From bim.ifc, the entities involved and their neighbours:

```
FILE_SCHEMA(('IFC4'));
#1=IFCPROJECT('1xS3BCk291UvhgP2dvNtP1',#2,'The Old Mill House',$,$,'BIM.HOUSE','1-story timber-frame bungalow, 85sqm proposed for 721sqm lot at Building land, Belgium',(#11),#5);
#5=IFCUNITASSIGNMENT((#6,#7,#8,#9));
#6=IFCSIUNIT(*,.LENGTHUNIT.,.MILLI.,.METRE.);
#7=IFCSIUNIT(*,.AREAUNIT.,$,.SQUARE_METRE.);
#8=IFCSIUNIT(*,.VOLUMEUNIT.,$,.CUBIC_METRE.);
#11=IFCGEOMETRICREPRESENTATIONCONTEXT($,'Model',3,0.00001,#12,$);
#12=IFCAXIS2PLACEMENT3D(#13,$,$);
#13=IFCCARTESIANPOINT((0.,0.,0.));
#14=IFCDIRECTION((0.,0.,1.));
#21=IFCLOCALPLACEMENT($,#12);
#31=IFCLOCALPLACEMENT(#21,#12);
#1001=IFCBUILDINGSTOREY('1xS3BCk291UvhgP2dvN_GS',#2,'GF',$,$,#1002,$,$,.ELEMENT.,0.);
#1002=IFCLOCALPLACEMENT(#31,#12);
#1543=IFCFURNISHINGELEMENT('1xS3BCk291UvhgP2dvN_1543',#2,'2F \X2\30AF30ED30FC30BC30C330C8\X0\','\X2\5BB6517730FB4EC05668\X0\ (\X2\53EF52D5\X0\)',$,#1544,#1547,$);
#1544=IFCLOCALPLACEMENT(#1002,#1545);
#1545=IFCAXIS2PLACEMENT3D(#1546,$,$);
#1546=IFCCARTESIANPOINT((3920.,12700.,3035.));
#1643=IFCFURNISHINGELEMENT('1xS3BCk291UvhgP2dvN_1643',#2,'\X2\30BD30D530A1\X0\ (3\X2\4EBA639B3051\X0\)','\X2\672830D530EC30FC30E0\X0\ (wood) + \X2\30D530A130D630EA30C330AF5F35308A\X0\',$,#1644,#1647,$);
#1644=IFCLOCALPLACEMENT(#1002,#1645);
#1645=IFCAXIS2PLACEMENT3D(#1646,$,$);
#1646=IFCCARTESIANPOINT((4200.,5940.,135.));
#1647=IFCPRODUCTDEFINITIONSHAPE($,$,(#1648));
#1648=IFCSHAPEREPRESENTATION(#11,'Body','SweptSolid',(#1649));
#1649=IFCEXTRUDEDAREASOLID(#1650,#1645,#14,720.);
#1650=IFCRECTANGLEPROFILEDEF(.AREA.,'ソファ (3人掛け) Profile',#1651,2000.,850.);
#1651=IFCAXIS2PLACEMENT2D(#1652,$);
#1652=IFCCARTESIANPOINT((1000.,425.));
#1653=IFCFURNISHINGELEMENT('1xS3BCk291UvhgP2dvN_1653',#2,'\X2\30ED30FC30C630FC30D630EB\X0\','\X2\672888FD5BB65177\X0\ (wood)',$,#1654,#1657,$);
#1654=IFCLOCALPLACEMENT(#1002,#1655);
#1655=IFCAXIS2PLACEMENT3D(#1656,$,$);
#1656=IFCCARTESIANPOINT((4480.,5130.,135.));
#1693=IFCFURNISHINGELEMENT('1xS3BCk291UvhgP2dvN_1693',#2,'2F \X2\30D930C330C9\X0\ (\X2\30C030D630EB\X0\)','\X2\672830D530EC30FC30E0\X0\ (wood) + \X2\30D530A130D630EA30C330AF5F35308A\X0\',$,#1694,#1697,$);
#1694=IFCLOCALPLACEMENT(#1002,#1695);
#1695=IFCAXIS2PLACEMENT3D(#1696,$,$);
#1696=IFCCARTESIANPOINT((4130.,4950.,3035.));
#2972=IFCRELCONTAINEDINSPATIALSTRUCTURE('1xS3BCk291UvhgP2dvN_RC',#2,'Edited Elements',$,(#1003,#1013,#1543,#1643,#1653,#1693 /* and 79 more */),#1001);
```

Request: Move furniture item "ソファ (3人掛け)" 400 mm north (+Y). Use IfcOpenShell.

```python
import ifcopenshell
import ifcopenshell.api.geometry
import ifcopenshell.util.placement
import ifcopenshell.util.unit

model = ifcopenshell.open("bim.ifc")
unit_scale = ifcopenshell.util.unit.calculate_unit_scale(model)

item = model.by_id(1643)
matrix = ifcopenshell.util.placement.get_local_placement(item.ObjectPlacement)
matrix[1, 3] += 0.4 / unit_scale
ifcopenshell.api.geometry.edit_object_placement(model, product=item, matrix=matrix, is_si=False)

print(ifcopenshell.util.placement.get_local_placement(item.ObjectPlacement).round(3) + 0.0)

model.write("bim_v2.ifc")
```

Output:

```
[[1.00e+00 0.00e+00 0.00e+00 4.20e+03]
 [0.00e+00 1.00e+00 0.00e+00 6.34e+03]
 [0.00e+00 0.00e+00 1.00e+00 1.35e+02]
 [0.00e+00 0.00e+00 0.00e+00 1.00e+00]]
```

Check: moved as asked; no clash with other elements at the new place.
